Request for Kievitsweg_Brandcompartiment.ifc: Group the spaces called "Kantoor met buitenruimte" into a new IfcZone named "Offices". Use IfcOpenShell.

First a look at what the model holds.

```python
import ifcopenshell

model = ifcopenshell.open("Kievitsweg_Brandcompartiment.ifc")
print(model.schema)
seen = {}
for space in model.by_type("IfcSpace"):
    seen[space.LongName] = seen.get(space.LongName, 0) + 1
for name, count in sorted(seen.items(), key=str):
    print(count, "x", name)
print("zones:", [z.Name for z in model.by_type("IfcZone")][:20])
```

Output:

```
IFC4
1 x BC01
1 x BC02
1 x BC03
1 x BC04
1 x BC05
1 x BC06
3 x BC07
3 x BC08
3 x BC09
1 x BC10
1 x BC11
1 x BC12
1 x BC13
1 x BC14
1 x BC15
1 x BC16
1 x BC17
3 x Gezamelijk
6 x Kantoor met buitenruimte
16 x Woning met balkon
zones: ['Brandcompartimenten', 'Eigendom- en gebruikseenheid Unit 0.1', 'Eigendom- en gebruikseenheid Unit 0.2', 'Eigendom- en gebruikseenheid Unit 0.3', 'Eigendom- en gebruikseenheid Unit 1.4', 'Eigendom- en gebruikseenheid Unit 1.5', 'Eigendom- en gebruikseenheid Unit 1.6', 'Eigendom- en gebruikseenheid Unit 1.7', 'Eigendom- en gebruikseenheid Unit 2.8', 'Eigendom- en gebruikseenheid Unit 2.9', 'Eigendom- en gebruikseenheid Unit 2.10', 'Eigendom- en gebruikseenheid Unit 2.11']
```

```python
import ifcopenshell
import ifcopenshell.api.group
import ifcopenshell.api.root

model = ifcopenshell.open("Kievitsweg_Brandcompartiment.ifc")

names = {"Kantoor met buitenruimte"}
spaces = [s for s in model.by_type("IfcSpace") if s.LongName in names]

zone = ifcopenshell.api.root.create_entity(model, ifc_class="IfcZone", name="Offices")
ifcopenshell.api.group.assign_group(model, products=spaces, group=zone)
print(len(spaces), "spaces in", zone.Name)

model.write("Kievitsweg_Brandcompartiment_edited.ifc")
```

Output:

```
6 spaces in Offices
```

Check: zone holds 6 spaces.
